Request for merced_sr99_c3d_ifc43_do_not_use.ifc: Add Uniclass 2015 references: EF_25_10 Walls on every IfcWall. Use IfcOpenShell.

First a look at what the model holds.

```python
import ifcopenshell

model = ifcopenshell.open("merced_sr99_c3d_ifc43_do_not_use.ifc")
print(model.schema)
print("classifications:", [c.Name for c in model.by_type("IfcClassification")])
for ifc_class in ("IfcDoor", "IfcRoof", "IfcStair", "IfcWall", "IfcWindow"):
    print(ifc_class, len(model.by_type(ifc_class)))
```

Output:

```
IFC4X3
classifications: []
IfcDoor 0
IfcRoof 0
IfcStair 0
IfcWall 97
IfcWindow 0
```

```python
import ifcopenshell
import ifcopenshell.api.classification

model = ifcopenshell.open("merced_sr99_c3d_ifc43_do_not_use.ifc")

system = ifcopenshell.api.classification.add_classification(model, classification="Uniclass 2015")

codes = {
    "IfcWall": ("EF_25_10", "Walls"),
}
for ifc_class, (code, name) in codes.items():
    products = model.by_type(ifc_class)
    ifcopenshell.api.classification.add_reference(
        model, products=products, classification=system, identification=code, name=name
    )
    print(code, len(products))

model.write("merced_sr99_c3d_ifc43_do_not_use_v2.ifc")
```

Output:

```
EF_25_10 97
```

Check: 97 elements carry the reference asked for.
